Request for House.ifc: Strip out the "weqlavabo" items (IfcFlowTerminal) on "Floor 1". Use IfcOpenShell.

First a look at what the model holds.

```python
import ifcopenshell
import ifcopenshell.util.element

model = ifcopenshell.open("House.ifc")
print(model.schema)
storey = next(s for s in model.by_type("IfcBuildingStorey") if s.Name == "Floor 1")
terminals = [e for e in ifcopenshell.util.element.get_decomposition(storey) if e.is_a("IfcFlowTerminal")]
seen = {}
for e in terminals:
    element_type = ifcopenshell.util.element.get_type(e)
    name = element_type.Name if element_type not in (None, e) else None
    seen[name] = seen.get(name, 0) + 1
for name, count in sorted(seen.items(), key=str):
    print(count, "x", name)
```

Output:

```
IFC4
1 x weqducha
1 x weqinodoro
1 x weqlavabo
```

```python
import ifcopenshell
import ifcopenshell.api.root
import ifcopenshell.util.element

model = ifcopenshell.open("House.ifc")

storey = next(s for s in model.by_type("IfcBuildingStorey") if s.Name == "Floor 1")
terminals = [e for e in ifcopenshell.util.element.get_decomposition(storey) if e.is_a("IfcFlowTerminal")]
targets = [e for e in terminals if (t := ifcopenshell.util.element.get_type(e)) not in (None, e) and t.Name == "weqlavabo"]

for e in targets:
    ifcopenshell.api.root.remove_product(model, product=e)
print(len(targets), "removed")

model.write("House-out.ifc")
```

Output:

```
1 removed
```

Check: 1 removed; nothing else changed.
